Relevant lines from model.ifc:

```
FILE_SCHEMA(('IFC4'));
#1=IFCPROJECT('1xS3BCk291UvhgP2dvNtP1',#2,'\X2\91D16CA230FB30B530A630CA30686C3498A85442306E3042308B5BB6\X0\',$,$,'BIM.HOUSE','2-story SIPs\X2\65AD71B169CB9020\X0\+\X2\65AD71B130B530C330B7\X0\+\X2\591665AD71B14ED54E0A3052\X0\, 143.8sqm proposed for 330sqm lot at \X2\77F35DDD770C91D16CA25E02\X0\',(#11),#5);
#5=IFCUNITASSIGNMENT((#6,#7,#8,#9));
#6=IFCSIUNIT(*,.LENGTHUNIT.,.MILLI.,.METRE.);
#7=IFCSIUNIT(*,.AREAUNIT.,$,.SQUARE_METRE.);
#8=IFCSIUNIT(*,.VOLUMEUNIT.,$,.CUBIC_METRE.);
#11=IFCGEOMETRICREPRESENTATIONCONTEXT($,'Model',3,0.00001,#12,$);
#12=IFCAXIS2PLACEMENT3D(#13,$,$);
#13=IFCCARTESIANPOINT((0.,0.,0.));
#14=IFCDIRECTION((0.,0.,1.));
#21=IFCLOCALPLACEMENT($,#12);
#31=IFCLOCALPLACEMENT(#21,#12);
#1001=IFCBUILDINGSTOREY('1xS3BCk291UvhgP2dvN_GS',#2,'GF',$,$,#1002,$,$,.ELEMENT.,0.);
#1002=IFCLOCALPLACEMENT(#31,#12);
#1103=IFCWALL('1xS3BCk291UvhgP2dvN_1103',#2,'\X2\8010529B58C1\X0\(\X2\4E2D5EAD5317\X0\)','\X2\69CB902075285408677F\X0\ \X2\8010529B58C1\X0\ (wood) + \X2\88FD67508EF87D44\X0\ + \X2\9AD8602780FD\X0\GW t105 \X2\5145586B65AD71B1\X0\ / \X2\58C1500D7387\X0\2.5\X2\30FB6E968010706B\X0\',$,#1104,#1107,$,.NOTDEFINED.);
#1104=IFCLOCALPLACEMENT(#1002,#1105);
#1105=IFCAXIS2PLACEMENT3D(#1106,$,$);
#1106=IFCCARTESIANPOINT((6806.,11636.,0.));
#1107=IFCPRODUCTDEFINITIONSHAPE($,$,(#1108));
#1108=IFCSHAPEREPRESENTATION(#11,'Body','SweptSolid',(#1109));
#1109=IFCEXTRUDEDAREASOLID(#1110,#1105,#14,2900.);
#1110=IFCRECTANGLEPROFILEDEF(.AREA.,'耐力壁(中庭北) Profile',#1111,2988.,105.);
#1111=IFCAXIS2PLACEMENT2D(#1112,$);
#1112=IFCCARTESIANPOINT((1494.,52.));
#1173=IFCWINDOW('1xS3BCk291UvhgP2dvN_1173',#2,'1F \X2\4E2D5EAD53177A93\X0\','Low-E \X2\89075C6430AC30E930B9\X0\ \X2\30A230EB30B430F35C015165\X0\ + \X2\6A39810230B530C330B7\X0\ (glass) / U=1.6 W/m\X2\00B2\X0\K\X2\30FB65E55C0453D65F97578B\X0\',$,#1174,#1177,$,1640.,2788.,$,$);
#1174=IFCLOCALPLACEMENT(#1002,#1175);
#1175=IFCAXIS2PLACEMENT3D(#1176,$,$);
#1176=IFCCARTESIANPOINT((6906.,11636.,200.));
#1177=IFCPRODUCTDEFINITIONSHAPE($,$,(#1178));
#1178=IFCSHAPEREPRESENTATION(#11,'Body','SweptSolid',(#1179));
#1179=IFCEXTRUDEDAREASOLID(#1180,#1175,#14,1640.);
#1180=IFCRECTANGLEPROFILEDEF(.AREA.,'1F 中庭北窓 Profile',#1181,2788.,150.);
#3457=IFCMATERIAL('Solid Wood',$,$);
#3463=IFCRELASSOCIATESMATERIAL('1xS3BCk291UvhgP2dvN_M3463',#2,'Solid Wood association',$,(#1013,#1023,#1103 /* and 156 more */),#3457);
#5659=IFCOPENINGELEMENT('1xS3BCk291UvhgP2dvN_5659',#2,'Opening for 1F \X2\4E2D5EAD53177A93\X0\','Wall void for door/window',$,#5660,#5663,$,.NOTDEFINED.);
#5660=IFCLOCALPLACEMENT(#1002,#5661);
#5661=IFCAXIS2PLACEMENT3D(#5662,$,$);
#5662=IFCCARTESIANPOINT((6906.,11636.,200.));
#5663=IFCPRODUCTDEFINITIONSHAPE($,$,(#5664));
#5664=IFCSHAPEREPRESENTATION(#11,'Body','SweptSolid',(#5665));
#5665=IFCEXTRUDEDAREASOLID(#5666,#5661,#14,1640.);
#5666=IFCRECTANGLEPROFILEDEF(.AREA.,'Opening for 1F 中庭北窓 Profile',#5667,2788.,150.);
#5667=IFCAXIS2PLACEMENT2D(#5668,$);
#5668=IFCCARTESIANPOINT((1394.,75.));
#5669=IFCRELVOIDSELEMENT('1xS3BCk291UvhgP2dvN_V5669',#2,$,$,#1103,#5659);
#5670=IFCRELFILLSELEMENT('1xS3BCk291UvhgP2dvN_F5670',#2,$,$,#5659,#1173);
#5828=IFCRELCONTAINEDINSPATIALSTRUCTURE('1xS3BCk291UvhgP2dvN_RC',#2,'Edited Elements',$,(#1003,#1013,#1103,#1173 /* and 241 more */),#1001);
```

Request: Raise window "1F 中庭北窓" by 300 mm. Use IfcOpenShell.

```python
import numpy as np
import ifcopenshell
import ifcopenshell.api.geometry
import ifcopenshell.util.placement
import ifcopenshell.util.unit

model = ifcopenshell.open("model.ifc")
unit_scale = ifcopenshell.util.unit.calculate_unit_scale(model)

window = model.by_id(1173)
opening = window.FillsVoids[0].RelatingOpeningElement
dz = 0.3 / unit_scale

shift = np.array([0.0, 0.0, dz])
# The window is not placed relative to its opening, so move both.
for product in (opening, window):
    matrix = ifcopenshell.util.placement.get_local_placement(product.ObjectPlacement)
    matrix[:3, 3] += shift
    ifcopenshell.api.geometry.edit_object_placement(model, product=product, matrix=matrix, is_si=False)

print(f"moved by {dz * unit_scale:+.3f} m")

model.write("model_edited.ifc")
```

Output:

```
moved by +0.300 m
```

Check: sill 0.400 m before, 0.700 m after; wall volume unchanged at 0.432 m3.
